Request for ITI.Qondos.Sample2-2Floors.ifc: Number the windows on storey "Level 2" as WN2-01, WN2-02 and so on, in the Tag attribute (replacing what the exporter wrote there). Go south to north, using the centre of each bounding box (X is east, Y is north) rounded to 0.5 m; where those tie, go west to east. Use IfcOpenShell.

First a look at what the model holds.

```python
import ifcopenshell
import ifcopenshell.util.element
import ifcopenshell.util.placement

model = ifcopenshell.open("ITI.Qondos.Sample2-2Floors.ifc")
print(model.schema)
storey = next(s for s in model.by_type("IfcBuildingStorey") if s.Name == "Level 2")
windows = [e for e in ifcopenshell.util.element.get_decomposition(storey) if e.is_a("IfcWindow")]
for e in sorted(windows, key=lambda e: e.id()):
    origin = ifcopenshell.util.placement.get_local_placement(e.ObjectPlacement)[:3, 3]
    print(e.id(), e.Tag, e.Name, origin.round(2) + 0.0, sep=" | ")
```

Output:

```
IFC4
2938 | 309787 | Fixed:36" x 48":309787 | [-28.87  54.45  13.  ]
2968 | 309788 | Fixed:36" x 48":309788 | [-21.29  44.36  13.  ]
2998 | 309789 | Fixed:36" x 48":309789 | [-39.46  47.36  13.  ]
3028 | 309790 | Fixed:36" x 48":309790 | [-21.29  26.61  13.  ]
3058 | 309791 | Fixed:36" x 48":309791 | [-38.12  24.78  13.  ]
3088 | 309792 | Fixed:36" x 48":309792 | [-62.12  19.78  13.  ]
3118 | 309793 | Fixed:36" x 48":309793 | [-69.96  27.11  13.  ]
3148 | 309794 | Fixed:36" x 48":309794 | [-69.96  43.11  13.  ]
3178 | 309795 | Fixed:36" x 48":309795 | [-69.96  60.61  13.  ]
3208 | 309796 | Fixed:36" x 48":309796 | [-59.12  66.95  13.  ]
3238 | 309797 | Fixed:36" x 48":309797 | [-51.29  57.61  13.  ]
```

```python
import ifcopenshell
import ifcopenshell.geom
import ifcopenshell.util.element
import ifcopenshell.util.shape

model = ifcopenshell.open("ITI.Qondos.Sample2-2Floors.ifc")
settings = ifcopenshell.geom.settings()
settings.set("use-world-coords", True)


def centre(element):
    shape = ifcopenshell.geom.create_shape(settings, element)
    return ifcopenshell.util.shape.get_bbox_centroid(shape.geometry)


storey = next(s for s in model.by_type("IfcBuildingStorey") if s.Name == "Level 2")
windows = [e for e in ifcopenshell.util.element.get_decomposition(storey) if e.is_a("IfcWindow")]

# Insertion points can sit at a corner or the storey origin, so sort by the geometry (in metres).
centres = {e: centre(e) for e in windows}
windows.sort(key=lambda e: (round(centres[e][1] / 0.5), centres[e][0]))

for i, e in enumerate(windows, start=1):
    number = f"WN2-{i:02d}"
    e.Tag = number
    print(e.id(), number)

model.write("ITI.Qondos.Sample2-2Floors_v2.ifc")
```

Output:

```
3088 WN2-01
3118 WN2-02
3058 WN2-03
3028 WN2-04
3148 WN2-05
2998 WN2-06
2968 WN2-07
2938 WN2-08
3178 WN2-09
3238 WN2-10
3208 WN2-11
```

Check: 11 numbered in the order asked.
